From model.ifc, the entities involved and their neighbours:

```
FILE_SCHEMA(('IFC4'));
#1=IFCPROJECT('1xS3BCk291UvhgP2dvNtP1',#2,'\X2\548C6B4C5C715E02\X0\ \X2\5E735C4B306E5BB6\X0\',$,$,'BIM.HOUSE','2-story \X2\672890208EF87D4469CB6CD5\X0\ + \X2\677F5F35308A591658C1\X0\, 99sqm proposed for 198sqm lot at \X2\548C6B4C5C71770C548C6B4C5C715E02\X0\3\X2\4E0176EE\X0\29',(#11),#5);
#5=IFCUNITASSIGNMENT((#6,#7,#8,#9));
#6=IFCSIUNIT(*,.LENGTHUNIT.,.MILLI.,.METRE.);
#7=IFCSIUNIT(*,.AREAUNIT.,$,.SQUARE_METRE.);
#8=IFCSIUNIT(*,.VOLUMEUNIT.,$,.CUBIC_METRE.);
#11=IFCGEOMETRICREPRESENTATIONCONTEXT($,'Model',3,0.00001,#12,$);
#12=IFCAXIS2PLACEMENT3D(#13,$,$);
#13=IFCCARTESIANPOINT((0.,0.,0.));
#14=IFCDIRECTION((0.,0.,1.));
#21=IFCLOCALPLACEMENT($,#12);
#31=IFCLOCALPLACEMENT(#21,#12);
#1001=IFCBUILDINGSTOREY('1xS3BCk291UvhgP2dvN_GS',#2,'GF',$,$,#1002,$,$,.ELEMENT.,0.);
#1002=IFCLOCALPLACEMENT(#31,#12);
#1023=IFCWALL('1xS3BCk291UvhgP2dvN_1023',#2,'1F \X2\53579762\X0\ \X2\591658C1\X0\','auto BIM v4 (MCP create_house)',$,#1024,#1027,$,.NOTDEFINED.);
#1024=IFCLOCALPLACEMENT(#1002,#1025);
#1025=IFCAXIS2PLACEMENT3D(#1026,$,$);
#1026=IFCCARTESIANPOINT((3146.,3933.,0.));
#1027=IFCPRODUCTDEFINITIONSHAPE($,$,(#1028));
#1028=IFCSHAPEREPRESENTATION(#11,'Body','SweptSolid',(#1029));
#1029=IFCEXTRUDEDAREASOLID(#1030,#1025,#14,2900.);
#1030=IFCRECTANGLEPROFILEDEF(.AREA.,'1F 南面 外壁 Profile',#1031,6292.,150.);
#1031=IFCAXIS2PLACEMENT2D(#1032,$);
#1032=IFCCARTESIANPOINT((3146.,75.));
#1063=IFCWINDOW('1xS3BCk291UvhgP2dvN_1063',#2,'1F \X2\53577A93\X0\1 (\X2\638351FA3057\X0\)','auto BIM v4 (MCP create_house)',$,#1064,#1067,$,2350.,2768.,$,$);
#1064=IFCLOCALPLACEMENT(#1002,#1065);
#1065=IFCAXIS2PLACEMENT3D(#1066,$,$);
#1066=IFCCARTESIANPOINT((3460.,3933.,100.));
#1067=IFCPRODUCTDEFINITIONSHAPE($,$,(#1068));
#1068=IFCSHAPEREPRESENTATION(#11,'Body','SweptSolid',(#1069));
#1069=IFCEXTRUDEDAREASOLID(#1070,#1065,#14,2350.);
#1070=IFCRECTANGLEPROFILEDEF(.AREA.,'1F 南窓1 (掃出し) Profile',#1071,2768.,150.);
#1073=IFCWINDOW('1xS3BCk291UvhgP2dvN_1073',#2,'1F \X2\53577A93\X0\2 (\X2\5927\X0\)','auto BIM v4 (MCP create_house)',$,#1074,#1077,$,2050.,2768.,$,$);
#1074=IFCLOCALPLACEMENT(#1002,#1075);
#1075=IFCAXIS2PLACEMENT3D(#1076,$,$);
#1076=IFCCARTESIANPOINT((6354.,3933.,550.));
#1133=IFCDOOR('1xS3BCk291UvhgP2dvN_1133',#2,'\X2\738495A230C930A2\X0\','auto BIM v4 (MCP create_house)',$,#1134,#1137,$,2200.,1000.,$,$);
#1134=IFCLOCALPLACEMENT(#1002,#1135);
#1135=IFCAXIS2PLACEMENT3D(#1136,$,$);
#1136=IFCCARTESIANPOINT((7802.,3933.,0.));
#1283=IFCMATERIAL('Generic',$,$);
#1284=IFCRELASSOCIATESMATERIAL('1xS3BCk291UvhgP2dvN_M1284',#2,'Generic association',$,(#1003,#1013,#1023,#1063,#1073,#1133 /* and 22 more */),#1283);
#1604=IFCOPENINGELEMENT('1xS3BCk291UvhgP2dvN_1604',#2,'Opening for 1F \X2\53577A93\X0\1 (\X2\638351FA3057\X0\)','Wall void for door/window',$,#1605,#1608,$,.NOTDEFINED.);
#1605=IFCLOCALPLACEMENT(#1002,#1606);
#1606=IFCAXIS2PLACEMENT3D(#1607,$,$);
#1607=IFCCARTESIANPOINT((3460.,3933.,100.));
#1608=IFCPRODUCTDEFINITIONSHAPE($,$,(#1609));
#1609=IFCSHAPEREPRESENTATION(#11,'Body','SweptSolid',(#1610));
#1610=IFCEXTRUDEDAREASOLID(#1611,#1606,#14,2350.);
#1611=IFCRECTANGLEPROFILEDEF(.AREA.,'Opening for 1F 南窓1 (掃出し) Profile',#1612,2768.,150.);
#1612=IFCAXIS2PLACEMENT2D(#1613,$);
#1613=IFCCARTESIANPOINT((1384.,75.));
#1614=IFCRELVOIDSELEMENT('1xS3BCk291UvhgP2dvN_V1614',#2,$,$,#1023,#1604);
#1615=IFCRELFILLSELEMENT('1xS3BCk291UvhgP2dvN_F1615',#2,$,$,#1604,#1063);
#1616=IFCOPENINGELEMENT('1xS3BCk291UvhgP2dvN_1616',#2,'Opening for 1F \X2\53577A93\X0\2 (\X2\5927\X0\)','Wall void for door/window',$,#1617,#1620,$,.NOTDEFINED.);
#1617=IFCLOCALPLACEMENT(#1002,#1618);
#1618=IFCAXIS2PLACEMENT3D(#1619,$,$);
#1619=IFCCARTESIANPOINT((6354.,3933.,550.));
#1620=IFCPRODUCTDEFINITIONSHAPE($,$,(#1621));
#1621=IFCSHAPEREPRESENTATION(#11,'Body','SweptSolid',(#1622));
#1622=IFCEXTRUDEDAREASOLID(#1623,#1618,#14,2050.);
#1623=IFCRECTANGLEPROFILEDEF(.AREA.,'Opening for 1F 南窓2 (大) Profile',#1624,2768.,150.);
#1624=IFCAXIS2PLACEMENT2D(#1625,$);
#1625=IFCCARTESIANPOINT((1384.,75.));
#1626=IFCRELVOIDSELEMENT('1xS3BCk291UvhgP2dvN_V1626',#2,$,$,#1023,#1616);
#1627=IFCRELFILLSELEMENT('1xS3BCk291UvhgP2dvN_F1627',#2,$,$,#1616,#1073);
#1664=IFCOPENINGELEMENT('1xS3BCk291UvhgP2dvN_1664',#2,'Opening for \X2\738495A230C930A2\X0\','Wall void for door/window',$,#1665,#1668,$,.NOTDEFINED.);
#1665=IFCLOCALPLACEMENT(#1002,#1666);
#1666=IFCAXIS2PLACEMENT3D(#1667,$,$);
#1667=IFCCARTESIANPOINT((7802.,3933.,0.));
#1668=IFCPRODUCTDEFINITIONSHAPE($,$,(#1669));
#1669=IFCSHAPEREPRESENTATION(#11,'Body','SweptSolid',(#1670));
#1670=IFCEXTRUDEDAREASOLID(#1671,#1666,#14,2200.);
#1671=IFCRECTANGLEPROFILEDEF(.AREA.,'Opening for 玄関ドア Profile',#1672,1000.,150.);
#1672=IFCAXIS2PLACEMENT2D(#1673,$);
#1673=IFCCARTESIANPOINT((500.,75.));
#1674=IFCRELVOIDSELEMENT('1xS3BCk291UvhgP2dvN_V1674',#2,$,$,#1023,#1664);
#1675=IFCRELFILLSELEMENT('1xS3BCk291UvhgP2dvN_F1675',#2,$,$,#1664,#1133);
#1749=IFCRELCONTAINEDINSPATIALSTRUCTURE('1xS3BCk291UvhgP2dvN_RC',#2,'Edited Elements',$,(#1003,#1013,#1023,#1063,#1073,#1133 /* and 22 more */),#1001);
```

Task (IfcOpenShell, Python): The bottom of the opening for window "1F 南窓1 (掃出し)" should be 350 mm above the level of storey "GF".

```python
import numpy as np
import ifcopenshell
import ifcopenshell.api.geometry
import ifcopenshell.geom
import ifcopenshell.util.element
import ifcopenshell.util.placement
import ifcopenshell.util.shape
import ifcopenshell.util.unit

model = ifcopenshell.open("model.ifc")
unit_scale = ifcopenshell.util.unit.calculate_unit_scale(model)

window = model.by_guid("1xS3BCk291UvhgP2dvN_1063")
opening = window.FillsVoids[0].RelatingOpeningElement
storey = ifcopenshell.util.element.get_container(window, ifc_class="IfcBuildingStorey")
level = ifcopenshell.util.placement.get_local_placement(storey.ObjectPlacement)[2, 3]

# The opening's origin need not be at the sill, so measure its lowest point.
shape = ifcopenshell.geom.create_shape(ifcopenshell.geom.settings(), opening)
bottom = ifcopenshell.util.shape.get_shape_bottom_elevation(shape, shape.geometry) / unit_scale
dz = level + 0.35 / unit_scale - bottom

shift = np.array([0.0, 0.0, dz])
# The window is not placed relative to its opening, so move both.
for product in (opening, window):
    matrix = ifcopenshell.util.placement.get_local_placement(product.ObjectPlacement)
    matrix[:3, 3] += shift
    ifcopenshell.api.geometry.edit_object_placement(model, product=product, matrix=matrix, is_si=False)

print(f"moved by {dz * unit_scale:+.3f} m")

model.write("model_v2.ifc")
```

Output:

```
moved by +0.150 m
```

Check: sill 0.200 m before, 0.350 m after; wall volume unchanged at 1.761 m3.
